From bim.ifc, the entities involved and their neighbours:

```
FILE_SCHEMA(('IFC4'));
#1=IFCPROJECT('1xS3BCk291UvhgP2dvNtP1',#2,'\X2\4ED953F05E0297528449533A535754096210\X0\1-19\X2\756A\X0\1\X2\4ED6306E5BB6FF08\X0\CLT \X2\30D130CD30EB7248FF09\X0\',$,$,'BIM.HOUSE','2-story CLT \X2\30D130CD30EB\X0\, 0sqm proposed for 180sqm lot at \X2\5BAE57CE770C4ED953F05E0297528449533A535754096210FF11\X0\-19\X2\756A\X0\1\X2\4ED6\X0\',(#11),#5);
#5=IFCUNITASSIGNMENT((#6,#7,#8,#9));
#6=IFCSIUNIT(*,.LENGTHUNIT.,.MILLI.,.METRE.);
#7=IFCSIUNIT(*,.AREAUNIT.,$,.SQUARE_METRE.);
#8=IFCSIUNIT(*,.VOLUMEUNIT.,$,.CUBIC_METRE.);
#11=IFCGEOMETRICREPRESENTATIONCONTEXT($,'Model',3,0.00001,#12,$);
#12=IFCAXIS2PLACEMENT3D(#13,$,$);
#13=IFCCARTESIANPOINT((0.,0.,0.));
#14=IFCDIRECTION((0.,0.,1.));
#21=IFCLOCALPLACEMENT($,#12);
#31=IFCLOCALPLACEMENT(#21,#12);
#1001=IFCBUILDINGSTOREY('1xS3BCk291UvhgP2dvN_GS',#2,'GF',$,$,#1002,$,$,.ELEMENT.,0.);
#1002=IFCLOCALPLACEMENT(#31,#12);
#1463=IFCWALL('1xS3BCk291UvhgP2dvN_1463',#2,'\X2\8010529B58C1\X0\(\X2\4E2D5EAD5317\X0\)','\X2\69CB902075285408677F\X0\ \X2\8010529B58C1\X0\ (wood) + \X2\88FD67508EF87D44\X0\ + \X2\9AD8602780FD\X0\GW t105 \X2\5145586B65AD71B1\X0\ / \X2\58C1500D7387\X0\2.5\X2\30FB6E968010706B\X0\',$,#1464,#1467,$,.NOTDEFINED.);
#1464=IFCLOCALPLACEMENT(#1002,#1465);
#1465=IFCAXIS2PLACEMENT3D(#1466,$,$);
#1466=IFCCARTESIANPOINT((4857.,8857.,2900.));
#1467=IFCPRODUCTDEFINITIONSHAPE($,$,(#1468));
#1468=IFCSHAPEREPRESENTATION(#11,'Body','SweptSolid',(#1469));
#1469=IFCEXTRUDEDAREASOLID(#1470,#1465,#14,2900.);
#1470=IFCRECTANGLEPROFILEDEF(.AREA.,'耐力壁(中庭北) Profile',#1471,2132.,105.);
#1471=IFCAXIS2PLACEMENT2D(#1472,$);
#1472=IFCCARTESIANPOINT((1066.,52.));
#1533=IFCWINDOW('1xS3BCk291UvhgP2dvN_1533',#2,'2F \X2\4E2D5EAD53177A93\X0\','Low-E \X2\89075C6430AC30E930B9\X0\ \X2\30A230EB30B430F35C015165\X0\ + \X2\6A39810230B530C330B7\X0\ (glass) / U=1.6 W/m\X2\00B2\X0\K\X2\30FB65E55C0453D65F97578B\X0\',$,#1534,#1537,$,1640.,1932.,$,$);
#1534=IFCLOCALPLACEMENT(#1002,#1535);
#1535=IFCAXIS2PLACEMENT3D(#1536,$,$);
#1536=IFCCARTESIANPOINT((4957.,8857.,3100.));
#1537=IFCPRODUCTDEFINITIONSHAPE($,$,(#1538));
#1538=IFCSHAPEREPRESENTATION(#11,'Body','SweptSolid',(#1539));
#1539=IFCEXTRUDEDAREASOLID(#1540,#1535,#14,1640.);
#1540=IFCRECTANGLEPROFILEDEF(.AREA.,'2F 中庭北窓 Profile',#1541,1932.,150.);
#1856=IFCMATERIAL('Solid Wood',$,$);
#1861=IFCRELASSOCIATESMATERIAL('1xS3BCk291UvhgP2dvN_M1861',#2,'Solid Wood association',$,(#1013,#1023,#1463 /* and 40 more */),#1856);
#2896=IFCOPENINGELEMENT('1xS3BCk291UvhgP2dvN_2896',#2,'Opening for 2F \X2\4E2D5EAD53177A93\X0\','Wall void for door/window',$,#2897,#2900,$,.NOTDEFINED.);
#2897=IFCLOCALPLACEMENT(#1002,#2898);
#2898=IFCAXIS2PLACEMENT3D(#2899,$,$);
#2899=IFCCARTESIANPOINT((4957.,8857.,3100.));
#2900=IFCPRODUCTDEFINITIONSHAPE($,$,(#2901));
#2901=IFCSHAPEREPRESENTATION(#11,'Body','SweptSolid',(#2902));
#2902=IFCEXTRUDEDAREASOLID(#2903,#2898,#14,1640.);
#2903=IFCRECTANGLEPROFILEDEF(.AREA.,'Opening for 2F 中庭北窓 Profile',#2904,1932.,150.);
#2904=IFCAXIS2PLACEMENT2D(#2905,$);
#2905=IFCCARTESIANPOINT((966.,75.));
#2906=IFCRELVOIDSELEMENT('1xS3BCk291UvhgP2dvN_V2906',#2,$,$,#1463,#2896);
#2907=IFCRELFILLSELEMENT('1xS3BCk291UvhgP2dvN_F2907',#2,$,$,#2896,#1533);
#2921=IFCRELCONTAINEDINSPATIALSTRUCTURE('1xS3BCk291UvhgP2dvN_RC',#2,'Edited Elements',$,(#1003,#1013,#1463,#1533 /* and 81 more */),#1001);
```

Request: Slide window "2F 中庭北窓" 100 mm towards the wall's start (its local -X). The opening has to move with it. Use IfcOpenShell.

```python
import ifcopenshell
import ifcopenshell.api.geometry
import ifcopenshell.util.placement
import ifcopenshell.util.unit

model = ifcopenshell.open("bim.ifc")
unit_scale = ifcopenshell.util.unit.calculate_unit_scale(model)

window = model.by_guid("1xS3BCk291UvhgP2dvN_1533")
opening = window.FillsVoids[0].RelatingOpeningElement
wall = opening.VoidsElements[0].RelatingBuildingElement

wall_matrix = ifcopenshell.util.placement.get_local_placement(wall.ObjectPlacement)
shift = wall_matrix[:3, 0] * -0.1 / unit_scale
before = ifcopenshell.util.placement.get_local_placement(window.ObjectPlacement)[:3, 3].copy()

# The window is not placed relative to its opening, so move both.
for product in (opening, window):
    matrix = ifcopenshell.util.placement.get_local_placement(product.ObjectPlacement)
    matrix[:3, 3] += shift
    ifcopenshell.api.geometry.edit_object_placement(model, product=product, matrix=matrix, is_si=False)

after = ifcopenshell.util.placement.get_local_placement(window.ObjectPlacement)[:3, 3]
print("window moved by", (after - before).round(3) + 0.0)

model.write("bim_v2.ifc")
```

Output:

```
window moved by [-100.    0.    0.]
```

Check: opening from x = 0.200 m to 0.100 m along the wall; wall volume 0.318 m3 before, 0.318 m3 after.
